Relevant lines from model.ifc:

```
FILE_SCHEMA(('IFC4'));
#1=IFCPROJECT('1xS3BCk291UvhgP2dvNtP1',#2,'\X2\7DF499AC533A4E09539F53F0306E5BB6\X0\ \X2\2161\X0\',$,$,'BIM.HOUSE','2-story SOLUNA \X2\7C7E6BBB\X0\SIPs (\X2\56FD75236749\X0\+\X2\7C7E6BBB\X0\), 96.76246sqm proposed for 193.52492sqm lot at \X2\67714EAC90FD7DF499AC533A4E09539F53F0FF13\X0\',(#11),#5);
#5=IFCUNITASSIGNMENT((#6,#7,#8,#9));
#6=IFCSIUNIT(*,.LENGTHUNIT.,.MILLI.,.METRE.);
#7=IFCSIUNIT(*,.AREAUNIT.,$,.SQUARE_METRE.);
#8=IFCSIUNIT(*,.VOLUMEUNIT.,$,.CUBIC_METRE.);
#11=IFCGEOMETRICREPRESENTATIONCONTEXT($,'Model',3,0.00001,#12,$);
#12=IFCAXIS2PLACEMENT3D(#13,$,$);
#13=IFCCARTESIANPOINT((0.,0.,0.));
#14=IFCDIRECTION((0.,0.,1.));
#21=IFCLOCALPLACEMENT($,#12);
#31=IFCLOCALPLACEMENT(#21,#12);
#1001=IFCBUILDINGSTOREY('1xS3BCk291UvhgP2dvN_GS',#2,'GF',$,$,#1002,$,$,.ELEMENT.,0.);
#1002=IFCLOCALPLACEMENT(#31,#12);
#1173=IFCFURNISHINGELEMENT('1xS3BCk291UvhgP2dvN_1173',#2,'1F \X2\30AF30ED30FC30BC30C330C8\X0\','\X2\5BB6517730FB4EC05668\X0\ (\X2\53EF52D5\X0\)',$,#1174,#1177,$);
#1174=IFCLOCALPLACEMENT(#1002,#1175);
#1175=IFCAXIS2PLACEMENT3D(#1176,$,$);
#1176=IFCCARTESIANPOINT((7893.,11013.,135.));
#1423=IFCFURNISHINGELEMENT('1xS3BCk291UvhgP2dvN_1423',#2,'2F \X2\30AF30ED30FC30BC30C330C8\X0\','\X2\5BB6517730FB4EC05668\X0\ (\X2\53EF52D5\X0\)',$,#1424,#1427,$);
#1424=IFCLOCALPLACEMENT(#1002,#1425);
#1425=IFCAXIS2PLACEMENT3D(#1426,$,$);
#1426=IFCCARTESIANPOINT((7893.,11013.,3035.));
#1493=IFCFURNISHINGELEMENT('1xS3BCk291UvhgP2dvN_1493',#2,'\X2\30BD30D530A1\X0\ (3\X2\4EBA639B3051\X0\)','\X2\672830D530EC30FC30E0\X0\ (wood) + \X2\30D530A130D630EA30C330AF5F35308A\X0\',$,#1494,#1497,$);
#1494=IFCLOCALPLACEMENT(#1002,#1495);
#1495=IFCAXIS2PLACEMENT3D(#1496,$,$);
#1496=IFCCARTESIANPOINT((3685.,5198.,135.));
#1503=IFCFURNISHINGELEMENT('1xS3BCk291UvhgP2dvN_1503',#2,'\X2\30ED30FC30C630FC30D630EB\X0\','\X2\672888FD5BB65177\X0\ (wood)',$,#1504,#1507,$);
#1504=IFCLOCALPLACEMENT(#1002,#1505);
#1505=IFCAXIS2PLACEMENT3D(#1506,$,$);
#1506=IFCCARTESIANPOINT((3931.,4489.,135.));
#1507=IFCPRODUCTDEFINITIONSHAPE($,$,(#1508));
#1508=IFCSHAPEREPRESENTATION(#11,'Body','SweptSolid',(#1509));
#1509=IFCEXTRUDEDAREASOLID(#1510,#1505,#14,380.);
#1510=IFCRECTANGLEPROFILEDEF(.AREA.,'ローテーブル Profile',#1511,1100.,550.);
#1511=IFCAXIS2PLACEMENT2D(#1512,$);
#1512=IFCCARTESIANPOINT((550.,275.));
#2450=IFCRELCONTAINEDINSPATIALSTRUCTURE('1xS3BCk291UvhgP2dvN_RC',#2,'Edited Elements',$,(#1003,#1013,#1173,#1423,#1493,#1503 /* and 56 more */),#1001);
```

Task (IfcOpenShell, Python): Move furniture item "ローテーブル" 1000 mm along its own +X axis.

```python
import ifcopenshell
import ifcopenshell.api.geometry
import ifcopenshell.util.placement
import ifcopenshell.util.unit

model = ifcopenshell.open("model.ifc")
unit_scale = ifcopenshell.util.unit.calculate_unit_scale(model)

item = model.by_id(1503)
matrix = ifcopenshell.util.placement.get_local_placement(item.ObjectPlacement)
matrix[:3, 3] += matrix[:3, 0] * 1 / unit_scale
ifcopenshell.api.geometry.edit_object_placement(model, product=item, matrix=matrix, is_si=False)

print(ifcopenshell.util.placement.get_local_placement(item.ObjectPlacement).round(3) + 0.0)

model.write("model_edited.ifc")
```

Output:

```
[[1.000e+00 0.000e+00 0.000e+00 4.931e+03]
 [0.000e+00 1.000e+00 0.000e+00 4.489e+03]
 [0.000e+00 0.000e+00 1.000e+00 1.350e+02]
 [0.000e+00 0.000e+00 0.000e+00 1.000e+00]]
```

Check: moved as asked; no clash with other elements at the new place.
